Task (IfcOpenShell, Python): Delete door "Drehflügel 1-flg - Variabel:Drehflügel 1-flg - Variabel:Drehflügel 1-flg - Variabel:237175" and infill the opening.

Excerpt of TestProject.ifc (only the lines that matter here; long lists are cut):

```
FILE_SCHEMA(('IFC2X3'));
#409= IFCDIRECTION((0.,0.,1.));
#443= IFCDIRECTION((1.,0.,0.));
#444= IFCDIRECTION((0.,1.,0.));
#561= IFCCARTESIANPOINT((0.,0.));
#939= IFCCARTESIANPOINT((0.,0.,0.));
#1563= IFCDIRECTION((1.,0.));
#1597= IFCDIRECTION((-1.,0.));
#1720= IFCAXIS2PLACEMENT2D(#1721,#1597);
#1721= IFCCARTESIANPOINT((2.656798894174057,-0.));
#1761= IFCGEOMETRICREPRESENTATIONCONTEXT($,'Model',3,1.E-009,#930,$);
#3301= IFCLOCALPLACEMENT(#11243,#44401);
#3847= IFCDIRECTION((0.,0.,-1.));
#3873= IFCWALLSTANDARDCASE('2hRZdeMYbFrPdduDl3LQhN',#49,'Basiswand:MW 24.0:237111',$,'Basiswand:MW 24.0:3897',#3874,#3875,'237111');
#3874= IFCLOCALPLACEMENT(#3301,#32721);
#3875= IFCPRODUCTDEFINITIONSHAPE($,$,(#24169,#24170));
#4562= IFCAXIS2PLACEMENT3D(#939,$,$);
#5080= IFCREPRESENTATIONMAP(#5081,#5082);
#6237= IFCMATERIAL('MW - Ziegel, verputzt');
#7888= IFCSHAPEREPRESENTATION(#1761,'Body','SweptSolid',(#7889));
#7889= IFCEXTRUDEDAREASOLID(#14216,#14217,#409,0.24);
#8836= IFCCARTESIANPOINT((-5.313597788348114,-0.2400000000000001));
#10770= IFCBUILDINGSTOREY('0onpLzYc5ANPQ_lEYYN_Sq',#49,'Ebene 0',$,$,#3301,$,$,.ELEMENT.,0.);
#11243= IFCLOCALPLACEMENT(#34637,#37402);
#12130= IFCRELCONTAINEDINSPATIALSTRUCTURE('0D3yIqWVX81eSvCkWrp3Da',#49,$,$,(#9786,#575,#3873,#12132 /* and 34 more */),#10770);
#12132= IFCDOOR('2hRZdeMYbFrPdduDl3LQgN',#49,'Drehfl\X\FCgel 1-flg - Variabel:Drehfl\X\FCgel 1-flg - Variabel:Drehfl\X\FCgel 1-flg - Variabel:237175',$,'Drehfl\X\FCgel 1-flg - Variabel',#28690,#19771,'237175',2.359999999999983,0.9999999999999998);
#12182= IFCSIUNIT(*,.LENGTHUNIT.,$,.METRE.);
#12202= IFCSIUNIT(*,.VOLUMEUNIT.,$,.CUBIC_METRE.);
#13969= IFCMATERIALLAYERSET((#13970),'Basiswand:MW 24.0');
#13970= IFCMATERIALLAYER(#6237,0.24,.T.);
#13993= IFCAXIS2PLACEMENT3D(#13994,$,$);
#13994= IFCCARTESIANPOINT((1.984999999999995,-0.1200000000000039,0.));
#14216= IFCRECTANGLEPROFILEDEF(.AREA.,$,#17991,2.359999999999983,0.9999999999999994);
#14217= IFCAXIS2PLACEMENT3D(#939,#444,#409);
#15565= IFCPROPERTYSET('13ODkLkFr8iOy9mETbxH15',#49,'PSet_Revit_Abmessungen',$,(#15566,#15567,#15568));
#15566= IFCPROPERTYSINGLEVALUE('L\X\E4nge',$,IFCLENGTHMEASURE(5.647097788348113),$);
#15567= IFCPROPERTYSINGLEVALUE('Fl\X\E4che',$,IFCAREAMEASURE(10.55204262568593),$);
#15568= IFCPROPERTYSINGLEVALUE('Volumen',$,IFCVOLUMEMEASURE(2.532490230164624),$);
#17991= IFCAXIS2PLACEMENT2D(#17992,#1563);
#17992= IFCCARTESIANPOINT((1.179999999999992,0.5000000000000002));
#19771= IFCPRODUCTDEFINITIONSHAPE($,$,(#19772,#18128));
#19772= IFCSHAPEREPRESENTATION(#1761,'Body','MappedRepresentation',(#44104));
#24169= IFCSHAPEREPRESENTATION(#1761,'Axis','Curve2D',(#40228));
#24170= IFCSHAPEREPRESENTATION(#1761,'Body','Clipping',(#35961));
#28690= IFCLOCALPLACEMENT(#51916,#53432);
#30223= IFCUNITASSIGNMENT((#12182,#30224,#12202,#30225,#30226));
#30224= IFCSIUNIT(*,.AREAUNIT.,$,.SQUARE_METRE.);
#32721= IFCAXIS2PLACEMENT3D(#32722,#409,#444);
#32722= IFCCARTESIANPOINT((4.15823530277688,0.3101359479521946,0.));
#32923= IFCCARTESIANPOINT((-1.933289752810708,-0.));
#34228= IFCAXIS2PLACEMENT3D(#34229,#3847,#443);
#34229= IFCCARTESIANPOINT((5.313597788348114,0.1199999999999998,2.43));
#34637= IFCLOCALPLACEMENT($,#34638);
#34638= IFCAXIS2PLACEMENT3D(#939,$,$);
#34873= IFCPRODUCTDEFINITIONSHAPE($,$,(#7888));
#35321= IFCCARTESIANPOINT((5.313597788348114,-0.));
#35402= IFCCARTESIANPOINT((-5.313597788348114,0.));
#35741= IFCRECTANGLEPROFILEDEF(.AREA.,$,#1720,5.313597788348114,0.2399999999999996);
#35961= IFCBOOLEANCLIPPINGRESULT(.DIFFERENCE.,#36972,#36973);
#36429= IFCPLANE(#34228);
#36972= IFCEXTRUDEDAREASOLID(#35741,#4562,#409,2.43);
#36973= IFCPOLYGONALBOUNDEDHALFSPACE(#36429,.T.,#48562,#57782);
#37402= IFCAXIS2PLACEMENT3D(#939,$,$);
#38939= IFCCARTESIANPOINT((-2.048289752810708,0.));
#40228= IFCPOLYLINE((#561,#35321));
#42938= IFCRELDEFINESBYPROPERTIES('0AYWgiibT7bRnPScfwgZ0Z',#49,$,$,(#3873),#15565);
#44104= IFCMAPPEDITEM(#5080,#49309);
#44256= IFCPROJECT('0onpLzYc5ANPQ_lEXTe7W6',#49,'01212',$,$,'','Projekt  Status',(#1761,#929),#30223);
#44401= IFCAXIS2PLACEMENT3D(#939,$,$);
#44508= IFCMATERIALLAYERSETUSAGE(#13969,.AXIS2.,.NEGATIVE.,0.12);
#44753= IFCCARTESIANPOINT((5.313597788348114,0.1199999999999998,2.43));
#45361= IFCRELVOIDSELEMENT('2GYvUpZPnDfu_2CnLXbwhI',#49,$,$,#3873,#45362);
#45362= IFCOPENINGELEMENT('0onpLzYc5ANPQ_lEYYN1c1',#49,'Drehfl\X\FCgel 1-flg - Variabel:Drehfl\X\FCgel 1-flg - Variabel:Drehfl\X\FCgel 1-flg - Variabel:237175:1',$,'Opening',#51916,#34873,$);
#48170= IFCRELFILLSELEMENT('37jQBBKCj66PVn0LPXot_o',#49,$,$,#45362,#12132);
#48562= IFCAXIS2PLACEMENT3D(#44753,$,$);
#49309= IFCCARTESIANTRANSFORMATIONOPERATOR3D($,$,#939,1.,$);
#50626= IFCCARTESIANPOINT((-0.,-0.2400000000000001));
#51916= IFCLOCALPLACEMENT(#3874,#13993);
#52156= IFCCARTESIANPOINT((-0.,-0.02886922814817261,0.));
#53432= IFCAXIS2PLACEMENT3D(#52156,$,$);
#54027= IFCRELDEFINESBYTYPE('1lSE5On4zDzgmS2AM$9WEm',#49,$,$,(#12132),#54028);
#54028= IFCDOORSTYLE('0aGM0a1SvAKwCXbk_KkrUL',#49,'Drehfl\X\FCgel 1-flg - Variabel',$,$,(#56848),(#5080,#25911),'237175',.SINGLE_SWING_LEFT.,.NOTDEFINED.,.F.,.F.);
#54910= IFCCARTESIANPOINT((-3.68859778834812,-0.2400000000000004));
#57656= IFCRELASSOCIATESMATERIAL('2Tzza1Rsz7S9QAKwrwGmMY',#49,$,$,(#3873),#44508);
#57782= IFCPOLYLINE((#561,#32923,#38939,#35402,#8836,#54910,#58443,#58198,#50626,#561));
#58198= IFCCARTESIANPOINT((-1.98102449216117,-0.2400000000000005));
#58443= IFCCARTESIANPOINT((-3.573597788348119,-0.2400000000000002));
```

```python
import ifcopenshell
import ifcopenshell.api.feature
import ifcopenshell.api.pset
import ifcopenshell.api.root
import ifcopenshell.geom
import ifcopenshell.util.element
import ifcopenshell.util.shape
import ifcopenshell.util.unit

model = ifcopenshell.open("TestProject.ifc")
area_scale = ifcopenshell.util.unit.calculate_unit_scale(model, "AREAUNIT")
volume_scale = ifcopenshell.util.unit.calculate_unit_scale(model, "VOLUMEUNIT")
settings = ifcopenshell.geom.settings()


def volume(element):
    """Net volume in cubic metres, openings subtracted."""
    shape = ifcopenshell.geom.create_shape(settings, element)
    return ifcopenshell.util.shape.get_volume(shape.geometry)


door = model.by_guid("2hRZdeMYbFrPdduDl3LQgN")
opening = door.FillsVoids[0].RelatingOpeningElement
wall = opening.VoidsElements[0].RelatingBuildingElement
before = volume(wall)

ifcopenshell.api.root.remove_product(model, product=door)
ifcopenshell.api.feature.remove_feature(model, feature=opening)

after = volume(wall)
thickness = 0.24  # wall thickness in metres

# Update the wall's stored quantities.
pset = model.by_id(ifcopenshell.util.element.get_pset(wall, "PSet_Revit_Abmessungen", should_inherit=False)["id"])
ifcopenshell.api.pset.edit_pset(model, pset=pset, properties={
    "Fläche": model.create_entity("IfcAreaMeasure", after / thickness / area_scale),
    "Volumen": model.create_entity("IfcVolumeMeasure", after / volume_scale),
})

print(f"wall volume {before:.3f} -> {after:.3f} m3")

model.write("TestProject_v2.ifc")
```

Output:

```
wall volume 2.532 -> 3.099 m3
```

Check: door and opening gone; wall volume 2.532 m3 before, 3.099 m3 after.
